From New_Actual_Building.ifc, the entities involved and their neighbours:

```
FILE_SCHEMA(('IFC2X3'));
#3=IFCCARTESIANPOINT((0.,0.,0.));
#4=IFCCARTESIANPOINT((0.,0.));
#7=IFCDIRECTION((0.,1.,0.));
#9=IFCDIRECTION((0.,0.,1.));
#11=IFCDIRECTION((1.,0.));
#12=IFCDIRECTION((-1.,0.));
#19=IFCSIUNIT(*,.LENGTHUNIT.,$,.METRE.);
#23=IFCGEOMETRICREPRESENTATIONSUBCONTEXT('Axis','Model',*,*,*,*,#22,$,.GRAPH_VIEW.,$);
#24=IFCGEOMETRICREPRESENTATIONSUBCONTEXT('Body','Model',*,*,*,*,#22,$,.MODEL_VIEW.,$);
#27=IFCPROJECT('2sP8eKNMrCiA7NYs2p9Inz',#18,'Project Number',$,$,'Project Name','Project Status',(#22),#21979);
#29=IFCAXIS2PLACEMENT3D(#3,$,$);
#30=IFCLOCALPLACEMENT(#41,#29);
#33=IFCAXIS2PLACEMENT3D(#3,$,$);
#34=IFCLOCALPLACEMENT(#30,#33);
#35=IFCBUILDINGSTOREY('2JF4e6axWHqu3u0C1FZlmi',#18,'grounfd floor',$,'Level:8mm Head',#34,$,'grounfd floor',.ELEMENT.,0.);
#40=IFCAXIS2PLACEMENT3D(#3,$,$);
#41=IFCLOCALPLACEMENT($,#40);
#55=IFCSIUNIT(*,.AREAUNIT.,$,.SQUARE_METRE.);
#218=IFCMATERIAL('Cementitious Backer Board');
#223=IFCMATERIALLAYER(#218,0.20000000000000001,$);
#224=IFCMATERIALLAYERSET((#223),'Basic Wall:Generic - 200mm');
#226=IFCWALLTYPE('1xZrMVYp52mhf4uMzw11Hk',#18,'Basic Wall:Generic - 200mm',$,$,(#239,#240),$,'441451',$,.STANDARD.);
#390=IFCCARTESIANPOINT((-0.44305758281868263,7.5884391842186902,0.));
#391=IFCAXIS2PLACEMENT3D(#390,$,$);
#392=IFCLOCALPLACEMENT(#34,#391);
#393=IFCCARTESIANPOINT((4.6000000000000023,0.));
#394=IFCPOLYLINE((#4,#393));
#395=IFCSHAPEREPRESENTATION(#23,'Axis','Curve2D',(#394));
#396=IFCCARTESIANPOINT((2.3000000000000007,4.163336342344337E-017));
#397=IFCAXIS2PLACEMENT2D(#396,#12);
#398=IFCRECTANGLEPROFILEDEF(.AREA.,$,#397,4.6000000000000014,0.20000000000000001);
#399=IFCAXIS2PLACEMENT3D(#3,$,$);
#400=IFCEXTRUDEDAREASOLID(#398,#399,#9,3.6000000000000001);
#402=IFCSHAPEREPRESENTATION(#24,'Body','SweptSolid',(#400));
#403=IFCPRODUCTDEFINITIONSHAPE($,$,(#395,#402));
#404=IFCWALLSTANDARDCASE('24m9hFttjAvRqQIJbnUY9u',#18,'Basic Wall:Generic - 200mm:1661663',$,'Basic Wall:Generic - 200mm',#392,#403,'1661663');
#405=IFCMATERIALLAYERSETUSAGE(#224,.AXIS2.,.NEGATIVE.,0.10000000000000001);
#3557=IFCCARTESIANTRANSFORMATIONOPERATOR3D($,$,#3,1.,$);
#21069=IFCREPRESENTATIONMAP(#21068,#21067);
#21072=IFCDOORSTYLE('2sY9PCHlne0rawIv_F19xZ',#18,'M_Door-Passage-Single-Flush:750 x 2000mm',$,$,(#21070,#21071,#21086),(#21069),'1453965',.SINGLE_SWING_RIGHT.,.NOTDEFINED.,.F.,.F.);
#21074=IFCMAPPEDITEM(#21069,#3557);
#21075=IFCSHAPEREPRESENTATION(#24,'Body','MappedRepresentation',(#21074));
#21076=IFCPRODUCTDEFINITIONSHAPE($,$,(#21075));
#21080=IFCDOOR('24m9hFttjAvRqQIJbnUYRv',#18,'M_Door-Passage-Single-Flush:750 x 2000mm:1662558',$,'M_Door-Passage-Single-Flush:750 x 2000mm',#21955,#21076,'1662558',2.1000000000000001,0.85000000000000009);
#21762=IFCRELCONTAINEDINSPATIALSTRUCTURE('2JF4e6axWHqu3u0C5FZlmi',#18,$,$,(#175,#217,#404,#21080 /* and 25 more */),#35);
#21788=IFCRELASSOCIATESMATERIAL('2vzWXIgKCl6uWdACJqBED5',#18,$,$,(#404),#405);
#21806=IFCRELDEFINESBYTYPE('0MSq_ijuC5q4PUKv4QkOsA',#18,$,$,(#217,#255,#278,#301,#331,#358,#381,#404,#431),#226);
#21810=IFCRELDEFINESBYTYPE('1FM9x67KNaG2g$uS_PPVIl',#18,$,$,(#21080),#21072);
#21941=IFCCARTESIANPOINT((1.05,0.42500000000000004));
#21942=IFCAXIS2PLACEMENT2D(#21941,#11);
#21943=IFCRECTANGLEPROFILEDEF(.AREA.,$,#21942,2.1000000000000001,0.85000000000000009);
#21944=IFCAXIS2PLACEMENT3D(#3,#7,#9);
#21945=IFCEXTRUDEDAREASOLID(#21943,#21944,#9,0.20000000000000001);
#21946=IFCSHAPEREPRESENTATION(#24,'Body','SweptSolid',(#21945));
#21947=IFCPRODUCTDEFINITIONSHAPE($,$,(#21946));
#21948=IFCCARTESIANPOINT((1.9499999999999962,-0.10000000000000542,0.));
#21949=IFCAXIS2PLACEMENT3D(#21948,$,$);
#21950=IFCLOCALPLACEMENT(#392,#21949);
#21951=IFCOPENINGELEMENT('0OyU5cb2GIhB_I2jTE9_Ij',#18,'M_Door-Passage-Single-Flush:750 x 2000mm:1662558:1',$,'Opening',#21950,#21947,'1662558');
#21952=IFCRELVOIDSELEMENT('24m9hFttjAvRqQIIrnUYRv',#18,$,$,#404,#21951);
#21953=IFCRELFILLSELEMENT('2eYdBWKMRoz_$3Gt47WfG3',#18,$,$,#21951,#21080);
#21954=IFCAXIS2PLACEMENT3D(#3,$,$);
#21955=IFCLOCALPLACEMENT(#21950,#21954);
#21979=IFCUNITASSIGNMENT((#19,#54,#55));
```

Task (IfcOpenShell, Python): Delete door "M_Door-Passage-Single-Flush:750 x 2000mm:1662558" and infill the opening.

```python
import ifcopenshell
import ifcopenshell.api.feature
import ifcopenshell.api.root
import ifcopenshell.geom
import ifcopenshell.util.shape

model = ifcopenshell.open("New_Actual_Building.ifc")
settings = ifcopenshell.geom.settings()


def volume(element):
    """Net volume in cubic metres, openings subtracted."""
    shape = ifcopenshell.geom.create_shape(settings, element)
    return ifcopenshell.util.shape.get_volume(shape.geometry)


door = model.by_guid("24m9hFttjAvRqQIJbnUYRv")
opening = door.FillsVoids[0].RelatingOpeningElement
wall = opening.VoidsElements[0].RelatingBuildingElement
before = volume(wall)

ifcopenshell.api.root.remove_product(model, product=door)
ifcopenshell.api.feature.remove_feature(model, feature=opening)

after = volume(wall)

print(f"wall volume {before:.3f} -> {after:.3f} m3")

model.write("New_Actual_Building_rev.ifc")
```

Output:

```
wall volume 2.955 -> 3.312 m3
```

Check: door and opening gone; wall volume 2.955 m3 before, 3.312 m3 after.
